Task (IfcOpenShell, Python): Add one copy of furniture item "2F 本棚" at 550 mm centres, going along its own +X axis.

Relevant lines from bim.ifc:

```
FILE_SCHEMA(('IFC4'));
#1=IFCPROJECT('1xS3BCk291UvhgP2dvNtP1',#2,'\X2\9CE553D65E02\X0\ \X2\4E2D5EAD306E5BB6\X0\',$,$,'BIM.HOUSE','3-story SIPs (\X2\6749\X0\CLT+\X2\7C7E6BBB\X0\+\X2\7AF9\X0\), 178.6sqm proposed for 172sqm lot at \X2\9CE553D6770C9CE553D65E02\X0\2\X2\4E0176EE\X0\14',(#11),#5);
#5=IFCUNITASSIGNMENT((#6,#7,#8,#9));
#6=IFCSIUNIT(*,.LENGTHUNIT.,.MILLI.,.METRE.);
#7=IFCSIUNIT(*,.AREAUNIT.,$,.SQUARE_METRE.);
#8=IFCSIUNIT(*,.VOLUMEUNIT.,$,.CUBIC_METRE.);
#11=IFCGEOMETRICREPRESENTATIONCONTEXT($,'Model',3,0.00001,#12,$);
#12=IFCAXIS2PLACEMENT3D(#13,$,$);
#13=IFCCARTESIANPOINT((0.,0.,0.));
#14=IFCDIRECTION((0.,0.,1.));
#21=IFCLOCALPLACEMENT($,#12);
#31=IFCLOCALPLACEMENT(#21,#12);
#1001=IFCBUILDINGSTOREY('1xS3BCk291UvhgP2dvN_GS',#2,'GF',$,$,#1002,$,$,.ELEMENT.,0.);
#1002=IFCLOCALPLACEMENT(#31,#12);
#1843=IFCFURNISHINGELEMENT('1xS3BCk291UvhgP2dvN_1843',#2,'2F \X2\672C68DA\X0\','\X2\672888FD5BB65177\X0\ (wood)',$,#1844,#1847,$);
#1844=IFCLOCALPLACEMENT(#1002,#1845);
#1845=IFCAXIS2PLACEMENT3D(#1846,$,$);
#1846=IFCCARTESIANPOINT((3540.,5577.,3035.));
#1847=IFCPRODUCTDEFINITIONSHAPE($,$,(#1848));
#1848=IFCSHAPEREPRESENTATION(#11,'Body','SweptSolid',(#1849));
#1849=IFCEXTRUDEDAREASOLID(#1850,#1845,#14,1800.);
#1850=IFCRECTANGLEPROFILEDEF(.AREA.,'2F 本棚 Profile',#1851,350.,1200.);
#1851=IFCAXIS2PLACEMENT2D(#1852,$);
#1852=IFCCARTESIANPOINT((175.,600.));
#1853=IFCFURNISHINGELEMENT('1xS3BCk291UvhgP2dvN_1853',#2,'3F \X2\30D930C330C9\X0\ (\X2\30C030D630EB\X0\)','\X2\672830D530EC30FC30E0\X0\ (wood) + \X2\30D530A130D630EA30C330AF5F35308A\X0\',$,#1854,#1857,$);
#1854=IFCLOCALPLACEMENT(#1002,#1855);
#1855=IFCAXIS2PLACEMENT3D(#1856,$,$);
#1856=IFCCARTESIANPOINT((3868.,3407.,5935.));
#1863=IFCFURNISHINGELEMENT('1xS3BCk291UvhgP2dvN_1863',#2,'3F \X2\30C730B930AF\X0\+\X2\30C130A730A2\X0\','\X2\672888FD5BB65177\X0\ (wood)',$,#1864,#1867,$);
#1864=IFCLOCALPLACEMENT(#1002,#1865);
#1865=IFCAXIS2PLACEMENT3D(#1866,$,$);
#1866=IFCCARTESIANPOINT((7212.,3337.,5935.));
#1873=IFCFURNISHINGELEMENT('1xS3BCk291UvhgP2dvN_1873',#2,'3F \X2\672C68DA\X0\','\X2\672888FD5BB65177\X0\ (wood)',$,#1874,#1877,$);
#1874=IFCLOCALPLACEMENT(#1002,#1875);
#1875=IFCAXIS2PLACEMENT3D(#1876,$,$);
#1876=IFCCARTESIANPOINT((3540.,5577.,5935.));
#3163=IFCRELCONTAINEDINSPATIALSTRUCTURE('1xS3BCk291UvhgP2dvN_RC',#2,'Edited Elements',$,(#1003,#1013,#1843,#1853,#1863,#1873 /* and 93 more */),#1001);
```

```python
import ifcopenshell
import ifcopenshell.api.geometry
import ifcopenshell.api.root
import ifcopenshell.util.element
import ifcopenshell.util.placement

model = ifcopenshell.open("bim.ifc")


def reuse_history(source, copy):
    """copy_class also copies each property set's owner history, people and application; keep the originals."""
    for rel in copy.IsDefinedBy:
        if rel.is_a("IfcRelDefinesByProperties") and (history := rel.RelatingPropertyDefinition.OwnerHistory):
            rel.RelatingPropertyDefinition.OwnerHistory = source.OwnerHistory
            ifcopenshell.util.element.remove_deep2(model, history)


source = model.by_guid("1xS3BCk291UvhgP2dvN_1843")
base = ifcopenshell.util.placement.get_local_placement(source.ObjectPlacement)
step = base[:3, 0] * 550.0

for i in range(1, 2):
    copy = ifcopenshell.api.root.copy_class(model, product=source)
    copy.Representation = ifcopenshell.util.element.copy_deep(
        model, source.Representation, exclude=["IfcGeometricRepresentationContext", "IfcRepresentationMap"]
    )
    reuse_history(source, copy)
    matrix = base.copy()
    matrix[:3, 3] += i * step
    print("added at", matrix[:3, 3].round(3) + 0.0)
    ifcopenshell.api.geometry.edit_object_placement(model, product=copy, matrix=matrix, is_si=False)

model.write("bim_rev.ifc")
```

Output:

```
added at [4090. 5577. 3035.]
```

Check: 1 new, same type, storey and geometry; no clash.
